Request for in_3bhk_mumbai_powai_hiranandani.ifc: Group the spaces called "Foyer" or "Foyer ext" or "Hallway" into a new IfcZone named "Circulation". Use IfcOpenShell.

First a look at what the model holds.

```python
import ifcopenshell

model = ifcopenshell.open("in_3bhk_mumbai_powai_hiranandani.ifc")
print(model.schema)
seen = {}
for space in model.by_type("IfcSpace"):
    seen[space.LongName] = seen.get(space.LongName, 0) + 1
for name, count in sorted(seen.items(), key=str):
    print(count, "x", name)
print("zones:", [z.Name for z in model.by_type("IfcZone")][:20])
```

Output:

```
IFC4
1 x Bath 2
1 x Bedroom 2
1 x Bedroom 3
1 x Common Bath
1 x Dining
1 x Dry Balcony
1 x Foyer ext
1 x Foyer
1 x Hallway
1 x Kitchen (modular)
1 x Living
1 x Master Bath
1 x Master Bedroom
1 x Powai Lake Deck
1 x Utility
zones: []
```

```python
import ifcopenshell
import ifcopenshell.api.group
import ifcopenshell.api.root

model = ifcopenshell.open("in_3bhk_mumbai_powai_hiranandani.ifc")

names = {"Foyer", "Foyer ext", "Hallway"}
spaces = [s for s in model.by_type("IfcSpace") if s.LongName in names]

zone = ifcopenshell.api.root.create_entity(model, ifc_class="IfcZone", name="Circulation")
ifcopenshell.api.group.assign_group(model, products=spaces, group=zone)
print(len(spaces), "spaces in", zone.Name)

model.write("in_3bhk_mumbai_powai_hiranandani-out.ifc")
```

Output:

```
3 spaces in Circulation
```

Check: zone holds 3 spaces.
